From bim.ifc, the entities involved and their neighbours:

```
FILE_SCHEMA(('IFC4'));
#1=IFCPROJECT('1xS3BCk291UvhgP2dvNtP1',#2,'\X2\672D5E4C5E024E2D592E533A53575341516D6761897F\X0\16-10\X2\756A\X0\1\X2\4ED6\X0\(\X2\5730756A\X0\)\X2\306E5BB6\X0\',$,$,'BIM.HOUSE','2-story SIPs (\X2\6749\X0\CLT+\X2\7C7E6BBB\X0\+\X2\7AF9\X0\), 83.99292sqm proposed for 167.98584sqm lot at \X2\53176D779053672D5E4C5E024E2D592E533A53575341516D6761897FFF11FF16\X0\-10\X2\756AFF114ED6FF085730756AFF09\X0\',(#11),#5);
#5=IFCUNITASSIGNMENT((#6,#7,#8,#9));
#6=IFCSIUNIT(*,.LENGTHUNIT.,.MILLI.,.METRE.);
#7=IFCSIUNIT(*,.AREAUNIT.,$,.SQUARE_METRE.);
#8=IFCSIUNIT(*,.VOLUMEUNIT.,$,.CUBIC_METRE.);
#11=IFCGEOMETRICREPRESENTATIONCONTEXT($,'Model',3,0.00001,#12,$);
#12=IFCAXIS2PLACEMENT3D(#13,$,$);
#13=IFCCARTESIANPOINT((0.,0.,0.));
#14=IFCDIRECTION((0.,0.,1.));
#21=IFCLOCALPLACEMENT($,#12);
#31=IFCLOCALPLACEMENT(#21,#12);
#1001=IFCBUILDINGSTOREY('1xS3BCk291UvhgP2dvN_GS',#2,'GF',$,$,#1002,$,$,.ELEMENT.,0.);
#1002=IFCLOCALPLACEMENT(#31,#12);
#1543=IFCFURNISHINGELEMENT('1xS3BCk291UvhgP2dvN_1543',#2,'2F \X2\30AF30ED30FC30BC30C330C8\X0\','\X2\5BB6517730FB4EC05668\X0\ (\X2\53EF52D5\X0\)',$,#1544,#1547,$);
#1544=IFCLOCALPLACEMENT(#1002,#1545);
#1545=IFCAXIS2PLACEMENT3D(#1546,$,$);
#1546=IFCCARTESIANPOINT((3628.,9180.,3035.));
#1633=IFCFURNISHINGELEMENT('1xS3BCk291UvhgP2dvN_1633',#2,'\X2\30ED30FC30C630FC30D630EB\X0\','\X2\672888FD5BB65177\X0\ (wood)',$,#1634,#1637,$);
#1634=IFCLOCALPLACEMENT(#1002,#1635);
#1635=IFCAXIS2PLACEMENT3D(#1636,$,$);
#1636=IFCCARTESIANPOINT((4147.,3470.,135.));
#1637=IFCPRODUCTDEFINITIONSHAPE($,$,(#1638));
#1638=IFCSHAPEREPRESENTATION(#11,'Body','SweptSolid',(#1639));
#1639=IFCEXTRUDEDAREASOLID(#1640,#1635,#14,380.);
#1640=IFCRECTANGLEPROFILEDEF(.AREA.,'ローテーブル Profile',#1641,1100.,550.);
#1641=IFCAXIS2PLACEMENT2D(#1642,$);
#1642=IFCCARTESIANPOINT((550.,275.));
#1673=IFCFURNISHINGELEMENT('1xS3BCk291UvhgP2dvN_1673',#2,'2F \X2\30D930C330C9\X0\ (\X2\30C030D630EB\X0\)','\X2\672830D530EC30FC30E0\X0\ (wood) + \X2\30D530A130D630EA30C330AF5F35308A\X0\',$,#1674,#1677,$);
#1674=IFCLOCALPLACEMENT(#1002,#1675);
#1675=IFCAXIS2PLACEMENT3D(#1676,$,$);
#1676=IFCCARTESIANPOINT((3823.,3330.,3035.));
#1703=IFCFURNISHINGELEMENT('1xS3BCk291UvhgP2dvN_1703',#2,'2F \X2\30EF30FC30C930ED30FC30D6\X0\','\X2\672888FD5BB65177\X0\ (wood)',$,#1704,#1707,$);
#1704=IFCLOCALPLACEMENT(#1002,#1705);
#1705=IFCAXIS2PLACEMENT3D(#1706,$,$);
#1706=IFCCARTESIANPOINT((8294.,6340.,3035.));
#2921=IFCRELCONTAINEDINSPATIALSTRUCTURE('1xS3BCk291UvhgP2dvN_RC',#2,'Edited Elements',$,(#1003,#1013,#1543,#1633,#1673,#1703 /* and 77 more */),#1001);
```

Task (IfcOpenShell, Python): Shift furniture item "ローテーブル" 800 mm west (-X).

```python
import ifcopenshell
import ifcopenshell.api.geometry
import ifcopenshell.util.placement

model = ifcopenshell.open("bim.ifc")

item = model.by_guid("1xS3BCk291UvhgP2dvN_1633")
matrix = ifcopenshell.util.placement.get_local_placement(item.ObjectPlacement)
matrix[0, 3] -= 800.0
ifcopenshell.api.geometry.edit_object_placement(model, product=item, matrix=matrix, is_si=False)

print(ifcopenshell.util.placement.get_local_placement(item.ObjectPlacement).round(3) + 0.0)

model.write("bim_edited.ifc")
```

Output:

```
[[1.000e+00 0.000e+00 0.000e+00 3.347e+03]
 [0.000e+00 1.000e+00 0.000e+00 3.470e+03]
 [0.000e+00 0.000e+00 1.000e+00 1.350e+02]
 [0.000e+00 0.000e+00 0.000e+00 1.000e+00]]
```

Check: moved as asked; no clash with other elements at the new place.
